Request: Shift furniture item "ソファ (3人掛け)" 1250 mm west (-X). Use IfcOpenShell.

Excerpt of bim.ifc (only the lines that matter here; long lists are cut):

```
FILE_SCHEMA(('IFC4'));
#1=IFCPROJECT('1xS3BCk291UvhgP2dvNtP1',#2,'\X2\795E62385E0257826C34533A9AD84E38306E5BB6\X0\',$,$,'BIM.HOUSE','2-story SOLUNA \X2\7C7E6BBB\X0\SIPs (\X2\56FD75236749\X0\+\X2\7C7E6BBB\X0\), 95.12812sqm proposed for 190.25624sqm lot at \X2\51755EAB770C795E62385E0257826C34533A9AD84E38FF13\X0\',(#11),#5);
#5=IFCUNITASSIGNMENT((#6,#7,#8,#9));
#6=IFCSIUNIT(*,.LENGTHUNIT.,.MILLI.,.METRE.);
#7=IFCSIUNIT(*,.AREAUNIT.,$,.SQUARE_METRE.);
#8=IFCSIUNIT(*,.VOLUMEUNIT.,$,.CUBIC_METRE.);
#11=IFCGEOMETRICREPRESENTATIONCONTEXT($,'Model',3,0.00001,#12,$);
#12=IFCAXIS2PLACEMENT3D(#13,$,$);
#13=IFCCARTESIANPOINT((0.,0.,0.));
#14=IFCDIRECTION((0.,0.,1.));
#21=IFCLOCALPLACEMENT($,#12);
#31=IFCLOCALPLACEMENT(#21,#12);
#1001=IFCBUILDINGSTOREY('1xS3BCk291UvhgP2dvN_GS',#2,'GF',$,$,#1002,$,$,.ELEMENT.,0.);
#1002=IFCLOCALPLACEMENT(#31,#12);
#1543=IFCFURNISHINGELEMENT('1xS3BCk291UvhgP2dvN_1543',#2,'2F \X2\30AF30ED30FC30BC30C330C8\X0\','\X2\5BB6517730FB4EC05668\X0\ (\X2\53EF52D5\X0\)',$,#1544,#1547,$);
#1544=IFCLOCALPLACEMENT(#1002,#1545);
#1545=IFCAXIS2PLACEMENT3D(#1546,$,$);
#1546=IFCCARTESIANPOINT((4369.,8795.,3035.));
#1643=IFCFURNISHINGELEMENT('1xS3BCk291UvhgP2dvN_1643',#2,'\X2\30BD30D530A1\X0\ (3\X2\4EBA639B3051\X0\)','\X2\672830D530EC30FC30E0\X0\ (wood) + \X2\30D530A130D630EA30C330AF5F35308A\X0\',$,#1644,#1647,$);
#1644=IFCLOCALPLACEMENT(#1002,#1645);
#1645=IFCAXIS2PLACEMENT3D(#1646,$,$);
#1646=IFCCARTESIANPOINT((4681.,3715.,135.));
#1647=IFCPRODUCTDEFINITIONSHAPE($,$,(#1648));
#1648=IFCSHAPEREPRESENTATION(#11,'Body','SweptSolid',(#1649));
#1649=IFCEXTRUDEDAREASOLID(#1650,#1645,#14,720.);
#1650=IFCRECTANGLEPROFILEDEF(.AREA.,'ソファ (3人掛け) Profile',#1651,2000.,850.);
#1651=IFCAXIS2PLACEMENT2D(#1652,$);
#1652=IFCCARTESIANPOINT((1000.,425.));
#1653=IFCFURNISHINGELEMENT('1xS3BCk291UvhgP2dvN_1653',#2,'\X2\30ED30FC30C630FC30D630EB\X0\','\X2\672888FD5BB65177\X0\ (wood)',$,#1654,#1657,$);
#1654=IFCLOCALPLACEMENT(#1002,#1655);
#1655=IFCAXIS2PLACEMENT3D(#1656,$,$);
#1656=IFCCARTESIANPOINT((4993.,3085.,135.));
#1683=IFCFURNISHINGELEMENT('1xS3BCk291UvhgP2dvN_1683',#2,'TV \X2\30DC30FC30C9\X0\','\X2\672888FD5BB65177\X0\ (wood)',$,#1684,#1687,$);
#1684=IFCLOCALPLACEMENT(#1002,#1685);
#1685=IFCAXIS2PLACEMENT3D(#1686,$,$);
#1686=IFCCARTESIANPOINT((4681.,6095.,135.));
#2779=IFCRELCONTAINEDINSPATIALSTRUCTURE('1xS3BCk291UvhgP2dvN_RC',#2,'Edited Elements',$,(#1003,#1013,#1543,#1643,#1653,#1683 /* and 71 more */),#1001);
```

```python
import ifcopenshell
import ifcopenshell.api.geometry
import ifcopenshell.util.placement

model = ifcopenshell.open("bim.ifc")

item = model.by_guid("1xS3BCk291UvhgP2dvN_1643")
matrix = ifcopenshell.util.placement.get_local_placement(item.ObjectPlacement)
matrix[0, 3] -= 1250.0
ifcopenshell.api.geometry.edit_object_placement(model, product=item, matrix=matrix, is_si=False)

print(ifcopenshell.util.placement.get_local_placement(item.ObjectPlacement).round(3) + 0.0)

model.write("bim-out.ifc")
```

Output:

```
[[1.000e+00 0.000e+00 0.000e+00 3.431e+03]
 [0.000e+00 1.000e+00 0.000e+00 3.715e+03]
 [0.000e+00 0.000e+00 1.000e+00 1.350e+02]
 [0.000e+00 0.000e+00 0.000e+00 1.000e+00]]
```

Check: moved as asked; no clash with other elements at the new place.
